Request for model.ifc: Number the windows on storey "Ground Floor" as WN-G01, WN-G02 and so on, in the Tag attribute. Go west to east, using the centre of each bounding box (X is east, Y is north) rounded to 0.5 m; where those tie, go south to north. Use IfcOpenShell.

First a look at what the model holds.

```python
import ifcopenshell
import ifcopenshell.util.element
import ifcopenshell.util.placement

model = ifcopenshell.open("model.ifc")
print(model.schema)
storey = next(s for s in model.by_type("IfcBuildingStorey") if s.Name == "Ground Floor")
windows = [e for e in ifcopenshell.util.element.get_decomposition(storey) if e.is_a("IfcWindow")]
for e in sorted(windows, key=lambda e: e.id()):
    origin = ifcopenshell.util.placement.get_local_placement(e.ObjectPlacement)[:3, 3]
    print(e.id(), e.Tag, e.Name, origin.round(2) + 0.0, sep=" | ")
```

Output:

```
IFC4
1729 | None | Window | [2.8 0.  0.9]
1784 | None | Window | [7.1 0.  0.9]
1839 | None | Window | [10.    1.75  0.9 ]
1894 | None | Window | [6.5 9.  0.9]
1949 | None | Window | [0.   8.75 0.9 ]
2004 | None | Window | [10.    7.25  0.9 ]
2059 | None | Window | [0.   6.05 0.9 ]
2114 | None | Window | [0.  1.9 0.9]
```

```python
import ifcopenshell
import ifcopenshell.geom
import ifcopenshell.util.element
import ifcopenshell.util.shape

model = ifcopenshell.open("model.ifc")
settings = ifcopenshell.geom.settings()
settings.set("use-world-coords", True)


def centre(element):
    shape = ifcopenshell.geom.create_shape(settings, element)
    return ifcopenshell.util.shape.get_bbox_centroid(shape.geometry)


storey = next(s for s in model.by_type("IfcBuildingStorey") if s.Name == "Ground Floor")
windows = [e for e in ifcopenshell.util.element.get_decomposition(storey) if e.is_a("IfcWindow")]

# Insertion points can sit at a corner or the storey origin, so sort by the geometry (in metres).
centres = {e: centre(e) for e in windows}
windows.sort(key=lambda e: (round(centres[e][0] / 0.5), centres[e][1]))

for i, e in enumerate(windows, start=1):
    number = f"WN-G{i:02d}"
    e.Tag = number
    print(e.id(), number)

model.write("model_updated.ifc")
```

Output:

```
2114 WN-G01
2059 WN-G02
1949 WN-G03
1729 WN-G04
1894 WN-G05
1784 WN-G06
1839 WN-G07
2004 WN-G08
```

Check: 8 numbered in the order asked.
